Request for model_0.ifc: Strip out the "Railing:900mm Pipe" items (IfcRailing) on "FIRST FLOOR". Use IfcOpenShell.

First a look at what the model holds.

```python
import ifcopenshell
import ifcopenshell.util.element

model = ifcopenshell.open("model_0.ifc")
print(model.schema)
storey = next(s for s in model.by_type("IfcBuildingStorey") if s.Name == "FIRST FLOOR")
railings = [e for e in ifcopenshell.util.element.get_decomposition(storey) if e.is_a("IfcRailing")]
seen = {}
for e in railings:
    element_type = ifcopenshell.util.element.get_type(e)
    name = element_type.Name if element_type not in (None, e) else None
    seen[name] = seen.get(name, 0) + 1
for name, count in sorted(seen.items(), key=str):
    print(count, "x", name)
```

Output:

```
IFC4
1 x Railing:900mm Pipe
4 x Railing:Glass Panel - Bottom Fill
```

```python
import ifcopenshell
import ifcopenshell.api.root
import ifcopenshell.util.element

model = ifcopenshell.open("model_0.ifc")

storey = next(s for s in model.by_type("IfcBuildingStorey") if s.Name == "FIRST FLOOR")
railings = [e for e in ifcopenshell.util.element.get_decomposition(storey) if e.is_a("IfcRailing")]
targets = [e for e in railings if (t := ifcopenshell.util.element.get_type(e)) not in (None, e) and t.Name == "Railing:900mm Pipe"]

for e in targets:
    ifcopenshell.api.root.remove_product(model, product=e)
print(len(targets), "removed")

model.write("model_0_v2.ifc")
```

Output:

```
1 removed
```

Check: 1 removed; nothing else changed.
